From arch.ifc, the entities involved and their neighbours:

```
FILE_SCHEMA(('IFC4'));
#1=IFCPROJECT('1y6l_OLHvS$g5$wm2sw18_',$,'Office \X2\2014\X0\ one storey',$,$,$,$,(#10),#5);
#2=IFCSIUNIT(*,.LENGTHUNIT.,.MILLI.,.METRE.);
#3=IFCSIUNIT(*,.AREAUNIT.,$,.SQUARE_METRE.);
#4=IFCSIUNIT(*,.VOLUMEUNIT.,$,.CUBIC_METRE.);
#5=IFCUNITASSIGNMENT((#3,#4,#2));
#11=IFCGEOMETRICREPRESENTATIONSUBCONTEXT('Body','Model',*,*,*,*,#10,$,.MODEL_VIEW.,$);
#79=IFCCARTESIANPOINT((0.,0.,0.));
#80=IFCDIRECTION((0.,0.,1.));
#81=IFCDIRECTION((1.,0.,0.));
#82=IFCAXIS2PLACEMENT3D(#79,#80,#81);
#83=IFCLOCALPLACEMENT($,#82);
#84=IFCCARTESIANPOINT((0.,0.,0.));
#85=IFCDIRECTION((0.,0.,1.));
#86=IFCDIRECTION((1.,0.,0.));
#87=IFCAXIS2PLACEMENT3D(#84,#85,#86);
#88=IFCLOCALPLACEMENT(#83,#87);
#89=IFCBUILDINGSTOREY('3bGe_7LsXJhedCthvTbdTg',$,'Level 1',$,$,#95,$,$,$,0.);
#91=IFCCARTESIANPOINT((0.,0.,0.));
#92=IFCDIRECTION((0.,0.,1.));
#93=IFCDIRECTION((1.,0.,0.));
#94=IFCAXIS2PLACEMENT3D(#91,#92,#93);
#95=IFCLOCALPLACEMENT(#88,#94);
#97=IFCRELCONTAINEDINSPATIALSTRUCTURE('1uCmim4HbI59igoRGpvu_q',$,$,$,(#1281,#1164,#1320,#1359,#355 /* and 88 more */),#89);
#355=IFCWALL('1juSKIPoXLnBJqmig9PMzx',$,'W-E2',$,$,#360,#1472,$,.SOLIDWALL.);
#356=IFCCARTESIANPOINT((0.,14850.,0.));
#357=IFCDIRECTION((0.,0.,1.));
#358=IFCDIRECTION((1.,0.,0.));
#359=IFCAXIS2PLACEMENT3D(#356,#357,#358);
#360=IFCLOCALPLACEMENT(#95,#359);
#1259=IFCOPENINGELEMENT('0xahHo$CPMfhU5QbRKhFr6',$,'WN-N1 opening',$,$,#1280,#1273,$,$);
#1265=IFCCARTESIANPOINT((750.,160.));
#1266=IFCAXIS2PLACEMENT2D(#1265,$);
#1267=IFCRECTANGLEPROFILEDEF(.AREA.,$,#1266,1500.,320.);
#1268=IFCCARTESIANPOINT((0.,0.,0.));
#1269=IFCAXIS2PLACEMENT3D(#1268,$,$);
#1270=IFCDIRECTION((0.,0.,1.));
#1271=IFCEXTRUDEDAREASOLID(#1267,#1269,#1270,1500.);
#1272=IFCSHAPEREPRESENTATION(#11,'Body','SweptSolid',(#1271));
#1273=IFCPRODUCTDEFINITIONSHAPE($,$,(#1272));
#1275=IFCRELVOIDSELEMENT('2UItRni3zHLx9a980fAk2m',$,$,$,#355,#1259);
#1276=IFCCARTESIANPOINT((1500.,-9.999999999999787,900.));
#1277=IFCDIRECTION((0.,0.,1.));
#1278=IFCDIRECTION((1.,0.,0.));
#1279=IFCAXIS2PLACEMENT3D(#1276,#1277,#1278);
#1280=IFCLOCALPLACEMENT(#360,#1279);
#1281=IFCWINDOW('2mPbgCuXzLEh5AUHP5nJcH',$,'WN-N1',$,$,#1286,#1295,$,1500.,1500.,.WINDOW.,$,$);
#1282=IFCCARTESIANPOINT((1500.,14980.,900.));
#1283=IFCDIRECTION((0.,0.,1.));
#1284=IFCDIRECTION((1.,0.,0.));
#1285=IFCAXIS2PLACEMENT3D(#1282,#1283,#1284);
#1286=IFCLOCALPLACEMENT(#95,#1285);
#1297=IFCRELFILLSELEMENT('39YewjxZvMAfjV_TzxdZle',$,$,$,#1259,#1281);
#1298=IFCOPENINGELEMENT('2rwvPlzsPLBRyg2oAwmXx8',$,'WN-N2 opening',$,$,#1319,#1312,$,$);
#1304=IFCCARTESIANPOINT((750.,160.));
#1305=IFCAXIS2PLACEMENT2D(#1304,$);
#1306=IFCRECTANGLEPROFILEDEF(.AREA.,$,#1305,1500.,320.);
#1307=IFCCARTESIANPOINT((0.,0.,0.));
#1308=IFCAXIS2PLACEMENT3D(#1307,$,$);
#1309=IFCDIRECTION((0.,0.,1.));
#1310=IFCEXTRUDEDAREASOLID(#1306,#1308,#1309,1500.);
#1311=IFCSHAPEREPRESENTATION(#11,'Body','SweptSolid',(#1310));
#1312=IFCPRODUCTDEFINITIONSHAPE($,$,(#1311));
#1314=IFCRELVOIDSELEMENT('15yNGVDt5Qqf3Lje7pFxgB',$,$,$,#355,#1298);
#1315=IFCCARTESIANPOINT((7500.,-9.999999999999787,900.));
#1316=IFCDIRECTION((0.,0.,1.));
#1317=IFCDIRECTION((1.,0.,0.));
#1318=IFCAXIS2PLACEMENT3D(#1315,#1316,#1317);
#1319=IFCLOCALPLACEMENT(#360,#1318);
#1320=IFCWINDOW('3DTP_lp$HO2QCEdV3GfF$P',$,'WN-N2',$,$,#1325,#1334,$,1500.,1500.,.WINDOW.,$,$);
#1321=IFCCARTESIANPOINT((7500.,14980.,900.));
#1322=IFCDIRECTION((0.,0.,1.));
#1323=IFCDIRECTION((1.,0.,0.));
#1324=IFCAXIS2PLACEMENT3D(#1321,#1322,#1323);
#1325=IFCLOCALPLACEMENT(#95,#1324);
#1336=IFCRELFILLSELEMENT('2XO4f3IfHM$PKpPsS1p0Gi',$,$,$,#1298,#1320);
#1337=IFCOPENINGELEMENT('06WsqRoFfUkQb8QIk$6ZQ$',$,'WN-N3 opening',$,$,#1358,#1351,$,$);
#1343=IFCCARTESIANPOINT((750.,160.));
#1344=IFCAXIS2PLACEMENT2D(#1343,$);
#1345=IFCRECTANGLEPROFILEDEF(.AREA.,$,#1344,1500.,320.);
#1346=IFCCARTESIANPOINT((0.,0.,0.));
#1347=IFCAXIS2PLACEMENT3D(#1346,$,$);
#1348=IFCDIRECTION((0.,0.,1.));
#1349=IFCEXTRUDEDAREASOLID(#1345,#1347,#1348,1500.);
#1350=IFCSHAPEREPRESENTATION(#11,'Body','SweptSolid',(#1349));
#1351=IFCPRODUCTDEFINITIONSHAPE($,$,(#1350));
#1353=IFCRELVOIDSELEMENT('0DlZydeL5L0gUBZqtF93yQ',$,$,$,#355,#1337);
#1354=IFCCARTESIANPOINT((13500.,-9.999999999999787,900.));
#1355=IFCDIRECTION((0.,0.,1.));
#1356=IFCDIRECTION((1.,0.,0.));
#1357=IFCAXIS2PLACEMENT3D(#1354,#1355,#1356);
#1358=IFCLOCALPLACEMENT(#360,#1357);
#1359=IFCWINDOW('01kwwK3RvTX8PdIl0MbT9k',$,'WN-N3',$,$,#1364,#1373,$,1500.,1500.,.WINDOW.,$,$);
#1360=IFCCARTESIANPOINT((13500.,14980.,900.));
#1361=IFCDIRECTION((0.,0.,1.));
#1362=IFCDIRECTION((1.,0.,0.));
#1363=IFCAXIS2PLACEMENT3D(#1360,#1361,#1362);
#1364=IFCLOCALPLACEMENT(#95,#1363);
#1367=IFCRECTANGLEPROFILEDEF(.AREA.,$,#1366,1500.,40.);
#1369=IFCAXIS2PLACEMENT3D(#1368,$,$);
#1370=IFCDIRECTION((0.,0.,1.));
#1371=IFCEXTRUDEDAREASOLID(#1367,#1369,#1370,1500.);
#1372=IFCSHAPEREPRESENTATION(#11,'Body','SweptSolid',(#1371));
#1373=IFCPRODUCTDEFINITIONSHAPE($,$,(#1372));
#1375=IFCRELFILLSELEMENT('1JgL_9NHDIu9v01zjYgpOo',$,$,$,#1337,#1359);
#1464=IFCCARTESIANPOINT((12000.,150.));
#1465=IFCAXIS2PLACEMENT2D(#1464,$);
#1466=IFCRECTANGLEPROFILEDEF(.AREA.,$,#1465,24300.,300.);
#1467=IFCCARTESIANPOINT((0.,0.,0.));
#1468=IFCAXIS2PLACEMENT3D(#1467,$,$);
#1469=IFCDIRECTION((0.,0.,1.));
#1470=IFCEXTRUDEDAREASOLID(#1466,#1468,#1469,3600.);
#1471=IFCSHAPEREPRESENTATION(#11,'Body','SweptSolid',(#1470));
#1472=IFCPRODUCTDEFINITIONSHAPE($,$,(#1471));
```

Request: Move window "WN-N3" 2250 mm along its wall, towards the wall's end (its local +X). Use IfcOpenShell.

```python
import ifcopenshell
import ifcopenshell.api.geometry
import ifcopenshell.util.placement
import ifcopenshell.util.unit

model = ifcopenshell.open("arch.ifc")
unit_scale = ifcopenshell.util.unit.calculate_unit_scale(model)

window = model.by_guid("01kwwK3RvTX8PdIl0MbT9k")
opening = window.FillsVoids[0].RelatingOpeningElement
wall = opening.VoidsElements[0].RelatingBuildingElement

wall_matrix = ifcopenshell.util.placement.get_local_placement(wall.ObjectPlacement)
shift = wall_matrix[:3, 0] * 2.25 / unit_scale
before = ifcopenshell.util.placement.get_local_placement(window.ObjectPlacement)[:3, 3].copy()

# The window is not placed relative to its opening, so move both.
for product in (opening, window):
    matrix = ifcopenshell.util.placement.get_local_placement(product.ObjectPlacement)
    matrix[:3, 3] += shift
    ifcopenshell.api.geometry.edit_object_placement(model, product=product, matrix=matrix, is_si=False)

after = ifcopenshell.util.placement.get_local_placement(window.ObjectPlacement)[:3, 3]
print("window moved by", (after - before).round(3) + 0.0)

model.write("arch-out.ifc")
```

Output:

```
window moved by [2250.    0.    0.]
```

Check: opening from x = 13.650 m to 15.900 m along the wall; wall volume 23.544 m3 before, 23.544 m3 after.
